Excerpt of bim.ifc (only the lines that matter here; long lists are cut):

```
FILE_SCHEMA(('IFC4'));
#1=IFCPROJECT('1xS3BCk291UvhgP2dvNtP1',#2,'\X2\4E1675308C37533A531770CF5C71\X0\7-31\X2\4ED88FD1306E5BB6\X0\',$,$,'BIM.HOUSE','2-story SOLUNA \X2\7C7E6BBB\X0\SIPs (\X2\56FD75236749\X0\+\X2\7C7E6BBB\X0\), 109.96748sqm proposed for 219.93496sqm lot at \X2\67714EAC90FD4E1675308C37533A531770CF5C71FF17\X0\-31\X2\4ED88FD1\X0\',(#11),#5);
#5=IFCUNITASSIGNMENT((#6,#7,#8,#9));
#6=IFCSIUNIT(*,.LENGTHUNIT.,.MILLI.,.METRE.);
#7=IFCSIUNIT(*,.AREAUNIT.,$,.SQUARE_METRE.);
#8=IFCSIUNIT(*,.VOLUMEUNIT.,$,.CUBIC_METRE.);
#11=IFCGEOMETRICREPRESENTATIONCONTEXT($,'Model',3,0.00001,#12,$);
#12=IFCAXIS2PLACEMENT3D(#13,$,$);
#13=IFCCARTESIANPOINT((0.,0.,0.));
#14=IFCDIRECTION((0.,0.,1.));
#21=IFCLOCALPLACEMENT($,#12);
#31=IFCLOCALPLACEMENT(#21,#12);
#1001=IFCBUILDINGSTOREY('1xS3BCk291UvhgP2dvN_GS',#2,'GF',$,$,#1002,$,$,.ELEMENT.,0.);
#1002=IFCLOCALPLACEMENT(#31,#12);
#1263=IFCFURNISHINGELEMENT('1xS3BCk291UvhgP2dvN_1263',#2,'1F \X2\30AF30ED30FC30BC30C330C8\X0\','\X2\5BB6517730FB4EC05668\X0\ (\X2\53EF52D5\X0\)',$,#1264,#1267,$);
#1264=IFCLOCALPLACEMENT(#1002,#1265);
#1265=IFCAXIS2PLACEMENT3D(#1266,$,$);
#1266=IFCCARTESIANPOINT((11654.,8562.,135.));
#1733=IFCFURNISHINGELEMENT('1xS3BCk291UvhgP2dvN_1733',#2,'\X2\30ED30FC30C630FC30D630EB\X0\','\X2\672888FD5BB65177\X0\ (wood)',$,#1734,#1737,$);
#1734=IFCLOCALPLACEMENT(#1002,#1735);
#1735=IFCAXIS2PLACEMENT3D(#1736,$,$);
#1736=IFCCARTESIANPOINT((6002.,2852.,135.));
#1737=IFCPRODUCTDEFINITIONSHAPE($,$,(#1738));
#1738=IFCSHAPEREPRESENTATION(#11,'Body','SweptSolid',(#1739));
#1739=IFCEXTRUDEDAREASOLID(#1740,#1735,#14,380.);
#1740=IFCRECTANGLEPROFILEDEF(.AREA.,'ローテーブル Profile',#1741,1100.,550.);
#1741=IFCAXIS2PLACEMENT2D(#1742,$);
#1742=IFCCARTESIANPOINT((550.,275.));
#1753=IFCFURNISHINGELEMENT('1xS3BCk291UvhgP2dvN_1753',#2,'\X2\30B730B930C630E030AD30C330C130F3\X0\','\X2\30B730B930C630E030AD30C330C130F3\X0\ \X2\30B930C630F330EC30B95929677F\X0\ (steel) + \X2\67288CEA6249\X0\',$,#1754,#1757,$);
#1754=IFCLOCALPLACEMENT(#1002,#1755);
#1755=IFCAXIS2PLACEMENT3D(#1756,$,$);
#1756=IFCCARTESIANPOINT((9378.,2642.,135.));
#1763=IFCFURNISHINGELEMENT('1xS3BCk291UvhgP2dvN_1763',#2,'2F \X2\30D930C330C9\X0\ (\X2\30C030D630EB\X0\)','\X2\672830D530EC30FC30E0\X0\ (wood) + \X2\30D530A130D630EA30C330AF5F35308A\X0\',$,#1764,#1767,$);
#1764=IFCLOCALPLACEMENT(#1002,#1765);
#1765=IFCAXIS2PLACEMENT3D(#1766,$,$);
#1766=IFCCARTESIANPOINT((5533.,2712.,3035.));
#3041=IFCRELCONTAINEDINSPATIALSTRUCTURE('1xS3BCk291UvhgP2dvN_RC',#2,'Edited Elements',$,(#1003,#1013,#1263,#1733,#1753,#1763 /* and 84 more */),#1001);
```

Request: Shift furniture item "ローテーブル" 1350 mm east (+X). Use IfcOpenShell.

```python
import ifcopenshell
import ifcopenshell.api.geometry
import ifcopenshell.util.placement
import ifcopenshell.util.unit

model = ifcopenshell.open("bim.ifc")
unit_scale = ifcopenshell.util.unit.calculate_unit_scale(model)

item = model.by_guid("1xS3BCk291UvhgP2dvN_1733")
matrix = ifcopenshell.util.placement.get_local_placement(item.ObjectPlacement)
matrix[0, 3] += 1.35 / unit_scale
ifcopenshell.api.geometry.edit_object_placement(model, product=item, matrix=matrix, is_si=False)

print(ifcopenshell.util.placement.get_local_placement(item.ObjectPlacement).round(3) + 0.0)

model.write("bim-out.ifc")
```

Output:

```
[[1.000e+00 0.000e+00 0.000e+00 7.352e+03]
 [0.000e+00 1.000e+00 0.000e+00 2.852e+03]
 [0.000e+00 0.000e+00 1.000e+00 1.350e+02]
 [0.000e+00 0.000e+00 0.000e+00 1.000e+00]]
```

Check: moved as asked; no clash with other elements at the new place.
